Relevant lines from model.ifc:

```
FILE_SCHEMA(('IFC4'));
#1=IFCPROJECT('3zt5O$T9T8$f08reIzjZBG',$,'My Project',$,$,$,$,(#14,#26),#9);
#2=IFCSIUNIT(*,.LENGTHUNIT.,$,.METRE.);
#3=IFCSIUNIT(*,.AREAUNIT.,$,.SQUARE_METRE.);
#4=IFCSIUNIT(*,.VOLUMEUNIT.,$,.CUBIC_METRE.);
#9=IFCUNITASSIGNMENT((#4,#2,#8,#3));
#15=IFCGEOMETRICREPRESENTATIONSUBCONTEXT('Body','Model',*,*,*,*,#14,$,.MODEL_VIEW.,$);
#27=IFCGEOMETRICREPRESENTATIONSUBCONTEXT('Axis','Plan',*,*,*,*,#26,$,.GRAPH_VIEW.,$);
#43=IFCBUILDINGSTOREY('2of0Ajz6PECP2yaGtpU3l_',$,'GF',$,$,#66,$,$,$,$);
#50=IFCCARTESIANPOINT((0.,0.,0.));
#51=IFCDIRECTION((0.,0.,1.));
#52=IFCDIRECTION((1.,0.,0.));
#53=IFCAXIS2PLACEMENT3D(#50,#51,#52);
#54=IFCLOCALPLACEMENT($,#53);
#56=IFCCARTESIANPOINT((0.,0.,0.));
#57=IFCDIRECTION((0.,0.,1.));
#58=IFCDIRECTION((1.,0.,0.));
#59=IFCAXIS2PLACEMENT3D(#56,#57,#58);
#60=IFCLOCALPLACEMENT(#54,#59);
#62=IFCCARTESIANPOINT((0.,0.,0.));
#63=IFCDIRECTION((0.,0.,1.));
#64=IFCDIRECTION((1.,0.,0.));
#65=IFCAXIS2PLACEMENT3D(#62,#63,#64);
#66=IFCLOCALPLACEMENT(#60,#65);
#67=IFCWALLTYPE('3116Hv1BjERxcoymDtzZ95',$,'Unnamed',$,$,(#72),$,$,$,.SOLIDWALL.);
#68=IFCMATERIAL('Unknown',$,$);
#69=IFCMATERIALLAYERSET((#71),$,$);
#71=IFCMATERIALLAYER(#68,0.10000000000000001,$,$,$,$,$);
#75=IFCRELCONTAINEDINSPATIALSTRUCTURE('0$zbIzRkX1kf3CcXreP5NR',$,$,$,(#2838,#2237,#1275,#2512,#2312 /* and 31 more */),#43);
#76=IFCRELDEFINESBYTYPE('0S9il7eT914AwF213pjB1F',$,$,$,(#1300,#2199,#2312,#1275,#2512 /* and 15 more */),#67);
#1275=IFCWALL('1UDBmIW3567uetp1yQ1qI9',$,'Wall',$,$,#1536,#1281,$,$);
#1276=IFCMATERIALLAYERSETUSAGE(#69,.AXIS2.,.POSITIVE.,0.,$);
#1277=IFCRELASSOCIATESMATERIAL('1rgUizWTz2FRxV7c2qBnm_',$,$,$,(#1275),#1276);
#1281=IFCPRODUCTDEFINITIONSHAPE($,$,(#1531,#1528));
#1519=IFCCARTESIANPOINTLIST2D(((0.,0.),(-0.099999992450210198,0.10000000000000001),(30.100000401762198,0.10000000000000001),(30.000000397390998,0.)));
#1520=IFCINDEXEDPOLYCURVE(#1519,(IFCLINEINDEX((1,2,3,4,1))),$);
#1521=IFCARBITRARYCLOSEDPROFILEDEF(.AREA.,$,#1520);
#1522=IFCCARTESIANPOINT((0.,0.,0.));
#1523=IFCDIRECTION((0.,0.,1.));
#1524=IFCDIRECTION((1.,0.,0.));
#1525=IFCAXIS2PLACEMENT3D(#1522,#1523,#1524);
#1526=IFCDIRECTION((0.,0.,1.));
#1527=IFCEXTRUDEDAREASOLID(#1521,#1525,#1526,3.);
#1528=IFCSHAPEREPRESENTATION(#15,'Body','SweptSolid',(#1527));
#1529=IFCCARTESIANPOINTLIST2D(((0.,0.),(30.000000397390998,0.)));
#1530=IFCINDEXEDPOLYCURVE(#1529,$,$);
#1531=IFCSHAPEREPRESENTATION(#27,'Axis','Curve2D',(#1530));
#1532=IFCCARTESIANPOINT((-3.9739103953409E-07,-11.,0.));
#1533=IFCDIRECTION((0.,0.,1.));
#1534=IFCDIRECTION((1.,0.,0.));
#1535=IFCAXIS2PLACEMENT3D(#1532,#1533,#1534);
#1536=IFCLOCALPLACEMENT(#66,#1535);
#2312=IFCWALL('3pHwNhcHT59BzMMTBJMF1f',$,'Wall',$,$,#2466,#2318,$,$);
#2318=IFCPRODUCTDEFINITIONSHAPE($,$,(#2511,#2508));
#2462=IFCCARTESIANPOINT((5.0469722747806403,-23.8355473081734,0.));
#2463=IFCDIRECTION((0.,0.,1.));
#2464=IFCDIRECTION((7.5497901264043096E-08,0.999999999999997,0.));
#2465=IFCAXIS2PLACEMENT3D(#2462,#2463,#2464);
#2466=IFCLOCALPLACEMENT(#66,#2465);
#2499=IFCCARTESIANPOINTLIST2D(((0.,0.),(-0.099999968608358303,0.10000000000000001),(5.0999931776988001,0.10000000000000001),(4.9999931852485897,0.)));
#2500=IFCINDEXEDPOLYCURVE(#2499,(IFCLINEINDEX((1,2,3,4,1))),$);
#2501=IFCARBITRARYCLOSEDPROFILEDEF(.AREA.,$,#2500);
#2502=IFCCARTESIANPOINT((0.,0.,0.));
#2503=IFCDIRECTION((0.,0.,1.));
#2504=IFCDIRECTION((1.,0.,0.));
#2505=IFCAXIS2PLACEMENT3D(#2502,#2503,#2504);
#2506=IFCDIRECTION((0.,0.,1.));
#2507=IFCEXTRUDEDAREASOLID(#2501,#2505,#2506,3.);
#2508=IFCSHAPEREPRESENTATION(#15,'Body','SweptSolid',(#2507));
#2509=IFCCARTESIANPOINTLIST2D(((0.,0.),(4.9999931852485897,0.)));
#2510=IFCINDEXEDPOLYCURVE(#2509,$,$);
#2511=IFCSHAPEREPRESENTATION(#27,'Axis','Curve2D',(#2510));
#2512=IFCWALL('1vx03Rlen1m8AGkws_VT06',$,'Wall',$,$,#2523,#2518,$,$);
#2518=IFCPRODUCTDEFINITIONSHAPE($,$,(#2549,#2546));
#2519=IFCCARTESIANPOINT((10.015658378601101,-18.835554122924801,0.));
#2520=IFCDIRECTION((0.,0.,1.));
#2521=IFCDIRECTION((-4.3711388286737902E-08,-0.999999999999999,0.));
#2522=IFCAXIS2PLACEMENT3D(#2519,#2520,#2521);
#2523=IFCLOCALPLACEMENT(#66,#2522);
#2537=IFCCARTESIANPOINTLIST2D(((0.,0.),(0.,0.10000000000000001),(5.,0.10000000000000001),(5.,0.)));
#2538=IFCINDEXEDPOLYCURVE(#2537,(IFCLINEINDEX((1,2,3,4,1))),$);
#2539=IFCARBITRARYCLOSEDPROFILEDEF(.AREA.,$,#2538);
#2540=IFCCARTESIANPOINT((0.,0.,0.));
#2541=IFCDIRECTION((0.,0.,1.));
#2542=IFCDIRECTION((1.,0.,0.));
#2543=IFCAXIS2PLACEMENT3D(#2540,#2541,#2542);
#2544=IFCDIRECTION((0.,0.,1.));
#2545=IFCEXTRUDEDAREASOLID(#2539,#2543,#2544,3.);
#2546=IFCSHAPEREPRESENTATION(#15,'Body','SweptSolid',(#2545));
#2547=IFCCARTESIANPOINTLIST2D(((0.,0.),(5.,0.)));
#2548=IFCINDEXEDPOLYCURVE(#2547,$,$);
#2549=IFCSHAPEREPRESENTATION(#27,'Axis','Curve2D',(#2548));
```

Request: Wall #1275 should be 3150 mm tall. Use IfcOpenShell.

```python
import ifcopenshell
import ifcopenshell.geom
import ifcopenshell.util.representation
import ifcopenshell.util.shape

model = ifcopenshell.open("model.ifc")
settings = ifcopenshell.geom.settings()


def volume(element):
    """Net volume in cubic metres, openings subtracted."""
    shape = ifcopenshell.geom.create_shape(settings, element)
    return ifcopenshell.util.shape.get_volume(shape.geometry)


wall = model.by_id(1275)
before = volume(wall)

body = ifcopenshell.util.representation.get_representation(wall, "Model", "Body")
solid = body.Items[0]
old_height = solid.Depth
solid.Depth = 3.15
after = volume(wall)

print(f"height {old_height:g} -> {solid.Depth:g}, volume {before:.3f} -> {after:.3f} m3")

model.write("model_v2.ifc")
```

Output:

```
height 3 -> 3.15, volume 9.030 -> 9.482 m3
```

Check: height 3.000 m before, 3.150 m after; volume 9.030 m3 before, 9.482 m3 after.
